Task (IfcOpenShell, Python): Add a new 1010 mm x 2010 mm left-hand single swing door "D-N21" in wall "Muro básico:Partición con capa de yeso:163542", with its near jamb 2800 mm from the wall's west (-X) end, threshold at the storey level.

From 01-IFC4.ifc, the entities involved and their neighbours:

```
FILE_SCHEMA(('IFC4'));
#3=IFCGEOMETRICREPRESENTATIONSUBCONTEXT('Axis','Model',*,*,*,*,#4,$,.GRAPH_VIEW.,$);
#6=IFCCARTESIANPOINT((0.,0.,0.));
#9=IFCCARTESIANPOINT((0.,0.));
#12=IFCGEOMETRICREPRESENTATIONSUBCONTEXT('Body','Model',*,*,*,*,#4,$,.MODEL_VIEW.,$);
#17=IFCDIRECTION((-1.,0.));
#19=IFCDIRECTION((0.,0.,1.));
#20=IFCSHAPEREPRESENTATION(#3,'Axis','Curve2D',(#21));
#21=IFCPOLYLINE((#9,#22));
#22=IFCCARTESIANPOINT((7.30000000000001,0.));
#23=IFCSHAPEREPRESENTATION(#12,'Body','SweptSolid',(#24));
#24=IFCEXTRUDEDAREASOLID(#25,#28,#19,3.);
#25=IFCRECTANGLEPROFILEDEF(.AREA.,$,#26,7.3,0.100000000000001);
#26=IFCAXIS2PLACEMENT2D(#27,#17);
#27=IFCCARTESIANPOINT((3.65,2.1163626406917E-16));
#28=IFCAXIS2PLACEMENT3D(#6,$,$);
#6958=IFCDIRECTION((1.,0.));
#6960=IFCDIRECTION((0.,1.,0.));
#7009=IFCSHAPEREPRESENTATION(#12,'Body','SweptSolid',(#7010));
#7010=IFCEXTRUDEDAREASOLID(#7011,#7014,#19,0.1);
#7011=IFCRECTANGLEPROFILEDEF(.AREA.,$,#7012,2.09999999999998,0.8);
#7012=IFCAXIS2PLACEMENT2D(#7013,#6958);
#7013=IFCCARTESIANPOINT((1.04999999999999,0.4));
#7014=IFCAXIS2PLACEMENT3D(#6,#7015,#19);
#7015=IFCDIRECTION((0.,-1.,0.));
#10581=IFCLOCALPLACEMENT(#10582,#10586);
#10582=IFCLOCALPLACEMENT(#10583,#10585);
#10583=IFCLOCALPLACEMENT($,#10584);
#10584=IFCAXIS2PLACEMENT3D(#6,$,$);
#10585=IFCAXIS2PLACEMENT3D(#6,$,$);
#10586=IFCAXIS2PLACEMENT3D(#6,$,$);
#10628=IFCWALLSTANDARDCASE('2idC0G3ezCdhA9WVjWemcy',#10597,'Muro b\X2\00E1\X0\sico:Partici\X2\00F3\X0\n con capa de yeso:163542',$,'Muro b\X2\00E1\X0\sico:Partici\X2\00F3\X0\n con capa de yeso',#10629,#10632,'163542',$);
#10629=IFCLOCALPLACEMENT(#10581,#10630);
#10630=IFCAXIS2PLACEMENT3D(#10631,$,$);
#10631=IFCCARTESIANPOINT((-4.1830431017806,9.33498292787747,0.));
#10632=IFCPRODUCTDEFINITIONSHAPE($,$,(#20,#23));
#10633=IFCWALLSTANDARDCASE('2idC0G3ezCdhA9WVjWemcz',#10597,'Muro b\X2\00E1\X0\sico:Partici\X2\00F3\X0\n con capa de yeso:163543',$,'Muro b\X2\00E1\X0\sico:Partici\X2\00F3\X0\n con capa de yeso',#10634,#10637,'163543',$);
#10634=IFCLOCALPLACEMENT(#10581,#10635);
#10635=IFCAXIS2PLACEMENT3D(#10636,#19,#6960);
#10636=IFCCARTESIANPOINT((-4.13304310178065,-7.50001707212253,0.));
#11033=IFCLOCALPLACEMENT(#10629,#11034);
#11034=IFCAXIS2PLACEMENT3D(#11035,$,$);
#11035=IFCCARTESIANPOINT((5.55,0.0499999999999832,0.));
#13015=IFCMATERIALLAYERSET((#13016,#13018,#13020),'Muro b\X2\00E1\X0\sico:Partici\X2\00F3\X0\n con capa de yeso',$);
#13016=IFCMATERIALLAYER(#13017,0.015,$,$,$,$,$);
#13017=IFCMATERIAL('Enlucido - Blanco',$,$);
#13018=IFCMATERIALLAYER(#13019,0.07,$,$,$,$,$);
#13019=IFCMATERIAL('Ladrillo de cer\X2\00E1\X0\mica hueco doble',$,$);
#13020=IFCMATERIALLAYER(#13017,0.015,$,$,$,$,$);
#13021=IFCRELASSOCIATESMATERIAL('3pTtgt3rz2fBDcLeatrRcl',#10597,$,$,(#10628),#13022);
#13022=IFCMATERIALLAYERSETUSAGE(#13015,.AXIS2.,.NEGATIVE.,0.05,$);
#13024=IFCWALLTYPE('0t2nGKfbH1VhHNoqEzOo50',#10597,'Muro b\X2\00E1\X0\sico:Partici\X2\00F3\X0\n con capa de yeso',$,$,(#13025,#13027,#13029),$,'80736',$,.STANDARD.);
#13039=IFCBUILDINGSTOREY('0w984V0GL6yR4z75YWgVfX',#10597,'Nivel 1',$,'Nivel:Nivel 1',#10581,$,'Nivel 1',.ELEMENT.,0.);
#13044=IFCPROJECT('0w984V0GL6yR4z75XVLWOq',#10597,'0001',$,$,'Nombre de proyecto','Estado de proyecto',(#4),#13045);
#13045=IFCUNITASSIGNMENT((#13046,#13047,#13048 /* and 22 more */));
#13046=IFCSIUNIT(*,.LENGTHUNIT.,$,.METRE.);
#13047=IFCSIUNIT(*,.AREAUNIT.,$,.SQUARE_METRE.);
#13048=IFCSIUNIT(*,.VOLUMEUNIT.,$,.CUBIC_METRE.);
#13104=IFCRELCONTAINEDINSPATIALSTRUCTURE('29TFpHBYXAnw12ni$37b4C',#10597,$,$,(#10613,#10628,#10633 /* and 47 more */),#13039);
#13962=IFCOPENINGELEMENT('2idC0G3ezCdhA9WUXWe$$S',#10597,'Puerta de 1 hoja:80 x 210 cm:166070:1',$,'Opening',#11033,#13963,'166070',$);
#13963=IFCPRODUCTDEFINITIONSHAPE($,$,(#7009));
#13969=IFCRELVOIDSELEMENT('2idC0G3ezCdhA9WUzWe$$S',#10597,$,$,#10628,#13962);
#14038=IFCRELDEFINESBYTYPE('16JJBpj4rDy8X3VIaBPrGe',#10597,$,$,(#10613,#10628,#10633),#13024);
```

```python
import numpy as np
import ifcopenshell
import ifcopenshell.api.feature
import ifcopenshell.api.geometry
import ifcopenshell.api.root
import ifcopenshell.api.spatial
import ifcopenshell.geom
import ifcopenshell.util.element
import ifcopenshell.util.placement
import ifcopenshell.util.representation
import ifcopenshell.util.shape
import ifcopenshell.util.unit

model = ifcopenshell.open("01-IFC4.ifc")
unit_scale = ifcopenshell.util.unit.calculate_unit_scale(model)
settings = ifcopenshell.geom.settings()


def volume(element):
    """Net volume in cubic metres, openings subtracted."""
    shape = ifcopenshell.geom.create_shape(settings, element)
    return ifcopenshell.util.shape.get_volume(shape.geometry)


wall = model.by_guid("2idC0G3ezCdhA9WVjWemcy")
storey = ifcopenshell.util.element.get_container(wall, ifc_class="IfcBuildingStorey")
context = ifcopenshell.util.representation.get_context(model, "Model", "Body", "MODEL_VIEW")
before = volume(wall)

width, height, from_end, sill = 1.01, 2.01, 2.8, 0.0  # metres

# The wall runs along its own X axis, and the end named is its -X end.
wall_shape = ifcopenshell.geom.create_shape(settings, wall)
x, y, z = ifcopenshell.util.shape.get_vertices(wall_shape.geometry).T
start = x.min() + from_end
face, thickness = float(y.min()), float(y.max() - y.min())
wall_matrix = ifcopenshell.util.placement.get_local_placement(wall.ObjectPlacement)
level = ifcopenshell.util.placement.get_local_placement(storey.ObjectPlacement)[2, 3]


def in_wall(x, y):
    """Placement at x, y metres in the wall's axes, at sill height."""
    matrix = wall_matrix.copy()
    matrix[:, 3] = wall_matrix @ np.array([x / unit_scale, y / unit_scale, 0.0, 1.0])
    matrix[2, 3] = level + sill / unit_scale
    return matrix


# Opening: a box that overshoots both wall faces by 50 mm.
opening = ifcopenshell.api.root.create_entity(model, ifc_class="IfcOpeningElement", predefined_type="OPENING")
box = ifcopenshell.api.geometry.add_wall_representation(
    model, context=context, length=width, height=height, thickness=thickness + 0.1
)
ifcopenshell.api.geometry.assign_representation(model, product=opening, representation=box)
ifcopenshell.api.geometry.edit_object_placement(model, product=opening, matrix=in_wall(start, face - 0.05), is_si=False)
ifcopenshell.api.feature.add_feature(model, feature=opening, element=wall)

door = ifcopenshell.api.root.create_entity(model, ifc_class="IfcDoor", name="D-N21", predefined_type="DOOR")
door.OverallWidth, door.OverallHeight = width / unit_scale, height / unit_scale
door.OperationType = "SINGLE_SWING_LEFT"
body = ifcopenshell.api.geometry.add_door_representation(
    model,
    context=context,
    overall_width=door.OverallWidth,
    overall_height=door.OverallHeight,
    operation_type="SINGLE_SWING_LEFT",
    lining_properties={"LiningDepth": thickness / unit_scale, "ThresholdDepth": thickness / unit_scale},
)
ifcopenshell.api.geometry.assign_representation(model, product=door, representation=body)
ifcopenshell.api.spatial.assign_container(model, products=[door], relating_structure=storey)
ifcopenshell.api.feature.add_filling(model, opening=opening, element=door)

# The lining spans the wall, so the door starts at the wall face.
ifcopenshell.api.geometry.edit_object_placement(model, product=door, matrix=in_wall(start, face), is_si=False)

after = volume(wall)

print(f"wall volume {before:.3f} -> {after:.3f} m3")

model.write("01-IFC4_rev.ifc")
```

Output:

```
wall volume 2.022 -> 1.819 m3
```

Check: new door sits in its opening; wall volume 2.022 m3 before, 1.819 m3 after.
